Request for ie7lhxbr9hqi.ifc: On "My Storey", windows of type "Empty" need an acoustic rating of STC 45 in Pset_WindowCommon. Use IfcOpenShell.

First a look at what the model holds.

```python
import ifcopenshell
import ifcopenshell.util.element

model = ifcopenshell.open("ie7lhxbr9hqi.ifc")
print(model.schema)
storey = next(s for s in model.by_type("IfcBuildingStorey") if s.Name == "My Storey")
windows = [e for e in ifcopenshell.util.element.get_decomposition(storey) if e.is_a("IfcWindow")]
seen = {}
for e in windows:
    element_type = ifcopenshell.util.element.get_type(e)
    key = (element_type.Name if element_type != e and element_type else None, ifcopenshell.util.element.get_pset(e, "Pset_WindowCommon", "AcousticRating"))
    seen[key] = seen.get(key, 0) + 1
for (name, value), count in sorted(seen.items(), key=str):
    print(count, "x", name, "|", value)
```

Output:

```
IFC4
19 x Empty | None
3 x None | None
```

```python
import ifcopenshell
import ifcopenshell.api.pset
import ifcopenshell.util.element

model = ifcopenshell.open("ie7lhxbr9hqi.ifc")

storey = next(s for s in model.by_type("IfcBuildingStorey") if s.Name == "My Storey")
windows = [e for e in ifcopenshell.util.element.get_decomposition(storey) if e.is_a("IfcWindow")]

count = 0
for e in windows:
    element_type = ifcopenshell.util.element.get_type(e)
    if element_type in (None, e) or element_type.Name != "Empty":
        continue
    # add_pset returns the element's existing set when there is one.
    pset = ifcopenshell.api.pset.add_pset(model, product=e, name="Pset_WindowCommon")
    ifcopenshell.api.pset.edit_pset(model, pset=pset, properties={"AcousticRating": "STC 45"})
    count += 1

print(count, "windows updated")

model.write("ie7lhxbr9hqi-out.ifc")
```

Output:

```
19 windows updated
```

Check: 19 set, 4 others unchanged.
